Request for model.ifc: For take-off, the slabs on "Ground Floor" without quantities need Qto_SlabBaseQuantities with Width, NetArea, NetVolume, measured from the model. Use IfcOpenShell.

First a look at what the model holds.

```python
import ifcopenshell
import ifcopenshell.util.element
import ifcopenshell.util.unit

model = ifcopenshell.open("model.ifc")
print(model.schema)
for unit_type in ("LENGTHUNIT", "AREAUNIT", "VOLUMEUNIT"):
    print(unit_type, ifcopenshell.util.unit.calculate_unit_scale(model, unit_type))
storey = next(s for s in model.by_type("IfcBuildingStorey") if s.Name == "Ground Floor")
slabs = [e for e in ifcopenshell.util.element.get_decomposition(storey) if e.is_a("IfcSlab")]
for e in sorted(slabs, key=lambda e: e.id()):
    print(e.id(), e.is_a(), e.Name, list(ifcopenshell.util.element.get_psets(e, qtos_only=True)), sep=" | ")
```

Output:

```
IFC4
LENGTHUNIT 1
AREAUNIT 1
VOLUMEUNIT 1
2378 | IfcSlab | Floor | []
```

```python
import ifcopenshell
import ifcopenshell.api.pset
import ifcopenshell.geom
import ifcopenshell.util.element
import ifcopenshell.util.shape
import ifcopenshell.util.unit

model = ifcopenshell.open("model.ifc")
unit_scale = ifcopenshell.util.unit.calculate_unit_scale(model)
area_scale = ifcopenshell.util.unit.calculate_unit_scale(model, "AREAUNIT")
volume_scale = ifcopenshell.util.unit.calculate_unit_scale(model, "VOLUMEUNIT")
settings = ifcopenshell.geom.settings()

storey = next(s for s in model.by_type("IfcBuildingStorey") if s.Name == "Ground Floor")
slabs = [e for e in ifcopenshell.util.element.get_decomposition(storey) if e.is_a("IfcSlab")]

for e in sorted(slabs, key=lambda e: e.id()):
    if ifcopenshell.util.element.get_psets(e, qtos_only=True, should_inherit=False):
        continue
    # Geometry comes back in metres, in the element's own axes.
    shape = ifcopenshell.geom.create_shape(settings, e)
    values = {
        "Width": ifcopenshell.util.shape.get_z(shape.geometry) / unit_scale,
        "NetArea": ifcopenshell.util.shape.get_footprint_area(shape.geometry) / area_scale,
        "NetVolume": ifcopenshell.util.shape.get_volume(shape.geometry) / volume_scale,
    }
    qto = ifcopenshell.api.pset.add_qto(model, product=e, name="Qto_SlabBaseQuantities")
    ifcopenshell.api.pset.edit_qto(model, qto=qto, properties=values)
    print(e.id(), {k: round(v, 3) for k, v in values.items()})

model.write("model_v2.ifc")
```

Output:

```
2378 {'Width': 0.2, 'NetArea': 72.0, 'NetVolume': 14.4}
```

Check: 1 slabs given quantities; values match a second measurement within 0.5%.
